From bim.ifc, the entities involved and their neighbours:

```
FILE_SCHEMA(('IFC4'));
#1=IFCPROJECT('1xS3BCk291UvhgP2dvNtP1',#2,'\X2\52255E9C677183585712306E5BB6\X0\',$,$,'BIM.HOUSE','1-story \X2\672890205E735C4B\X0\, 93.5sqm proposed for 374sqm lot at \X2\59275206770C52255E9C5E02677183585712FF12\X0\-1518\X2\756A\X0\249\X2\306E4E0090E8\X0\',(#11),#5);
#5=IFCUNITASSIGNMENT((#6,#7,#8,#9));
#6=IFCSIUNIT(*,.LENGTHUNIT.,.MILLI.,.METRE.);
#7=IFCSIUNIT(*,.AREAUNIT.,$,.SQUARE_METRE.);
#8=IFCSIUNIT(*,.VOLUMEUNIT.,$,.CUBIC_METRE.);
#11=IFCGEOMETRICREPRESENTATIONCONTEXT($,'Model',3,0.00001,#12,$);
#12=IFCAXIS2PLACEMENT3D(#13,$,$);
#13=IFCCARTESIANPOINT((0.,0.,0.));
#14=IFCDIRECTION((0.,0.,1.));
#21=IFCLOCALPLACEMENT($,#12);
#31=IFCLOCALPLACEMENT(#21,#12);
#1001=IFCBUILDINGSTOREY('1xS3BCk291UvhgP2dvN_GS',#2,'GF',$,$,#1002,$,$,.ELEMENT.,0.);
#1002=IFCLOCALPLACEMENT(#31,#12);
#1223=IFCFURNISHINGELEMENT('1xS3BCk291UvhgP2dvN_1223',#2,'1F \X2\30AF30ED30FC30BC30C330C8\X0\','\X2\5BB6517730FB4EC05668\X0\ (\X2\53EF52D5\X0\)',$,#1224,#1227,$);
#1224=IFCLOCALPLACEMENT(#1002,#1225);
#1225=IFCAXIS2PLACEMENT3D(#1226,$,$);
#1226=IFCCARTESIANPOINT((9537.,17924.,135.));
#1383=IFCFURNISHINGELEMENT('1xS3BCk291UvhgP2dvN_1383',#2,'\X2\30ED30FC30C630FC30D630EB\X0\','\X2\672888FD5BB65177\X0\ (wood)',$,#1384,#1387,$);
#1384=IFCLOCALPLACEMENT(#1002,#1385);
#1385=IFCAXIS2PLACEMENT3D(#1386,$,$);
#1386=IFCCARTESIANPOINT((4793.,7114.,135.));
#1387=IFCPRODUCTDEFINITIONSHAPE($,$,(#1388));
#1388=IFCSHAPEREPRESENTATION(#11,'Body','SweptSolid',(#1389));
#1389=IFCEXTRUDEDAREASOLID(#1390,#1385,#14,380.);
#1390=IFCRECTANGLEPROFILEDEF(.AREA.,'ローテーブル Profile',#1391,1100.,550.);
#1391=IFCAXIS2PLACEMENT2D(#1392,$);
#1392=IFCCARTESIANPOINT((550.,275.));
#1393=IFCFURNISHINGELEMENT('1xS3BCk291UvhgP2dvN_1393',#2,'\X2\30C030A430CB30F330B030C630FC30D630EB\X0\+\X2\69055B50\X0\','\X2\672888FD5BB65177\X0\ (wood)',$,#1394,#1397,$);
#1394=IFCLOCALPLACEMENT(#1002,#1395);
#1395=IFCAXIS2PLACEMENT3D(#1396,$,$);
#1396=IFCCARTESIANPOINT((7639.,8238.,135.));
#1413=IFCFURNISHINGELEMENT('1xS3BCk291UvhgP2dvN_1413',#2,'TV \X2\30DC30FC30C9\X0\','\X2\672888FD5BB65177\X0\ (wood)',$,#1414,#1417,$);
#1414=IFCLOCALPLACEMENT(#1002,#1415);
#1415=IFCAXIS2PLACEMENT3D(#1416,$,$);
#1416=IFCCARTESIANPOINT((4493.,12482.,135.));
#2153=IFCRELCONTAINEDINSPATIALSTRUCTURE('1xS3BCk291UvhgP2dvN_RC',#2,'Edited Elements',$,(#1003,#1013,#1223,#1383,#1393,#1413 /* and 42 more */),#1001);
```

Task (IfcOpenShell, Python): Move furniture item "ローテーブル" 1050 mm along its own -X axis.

```python
import ifcopenshell
import ifcopenshell.api.geometry
import ifcopenshell.util.placement
import ifcopenshell.util.unit

model = ifcopenshell.open("bim.ifc")
unit_scale = ifcopenshell.util.unit.calculate_unit_scale(model)

item = model.by_id(1383)
matrix = ifcopenshell.util.placement.get_local_placement(item.ObjectPlacement)
matrix[:3, 3] -= matrix[:3, 0] * 1.05 / unit_scale
ifcopenshell.api.geometry.edit_object_placement(model, product=item, matrix=matrix, is_si=False)

print(ifcopenshell.util.placement.get_local_placement(item.ObjectPlacement).round(3) + 0.0)

model.write("bim_edited.ifc")
```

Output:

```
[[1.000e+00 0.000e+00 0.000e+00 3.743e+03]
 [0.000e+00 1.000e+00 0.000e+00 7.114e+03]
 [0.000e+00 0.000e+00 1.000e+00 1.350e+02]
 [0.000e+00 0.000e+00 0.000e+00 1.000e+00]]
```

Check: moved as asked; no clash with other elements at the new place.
